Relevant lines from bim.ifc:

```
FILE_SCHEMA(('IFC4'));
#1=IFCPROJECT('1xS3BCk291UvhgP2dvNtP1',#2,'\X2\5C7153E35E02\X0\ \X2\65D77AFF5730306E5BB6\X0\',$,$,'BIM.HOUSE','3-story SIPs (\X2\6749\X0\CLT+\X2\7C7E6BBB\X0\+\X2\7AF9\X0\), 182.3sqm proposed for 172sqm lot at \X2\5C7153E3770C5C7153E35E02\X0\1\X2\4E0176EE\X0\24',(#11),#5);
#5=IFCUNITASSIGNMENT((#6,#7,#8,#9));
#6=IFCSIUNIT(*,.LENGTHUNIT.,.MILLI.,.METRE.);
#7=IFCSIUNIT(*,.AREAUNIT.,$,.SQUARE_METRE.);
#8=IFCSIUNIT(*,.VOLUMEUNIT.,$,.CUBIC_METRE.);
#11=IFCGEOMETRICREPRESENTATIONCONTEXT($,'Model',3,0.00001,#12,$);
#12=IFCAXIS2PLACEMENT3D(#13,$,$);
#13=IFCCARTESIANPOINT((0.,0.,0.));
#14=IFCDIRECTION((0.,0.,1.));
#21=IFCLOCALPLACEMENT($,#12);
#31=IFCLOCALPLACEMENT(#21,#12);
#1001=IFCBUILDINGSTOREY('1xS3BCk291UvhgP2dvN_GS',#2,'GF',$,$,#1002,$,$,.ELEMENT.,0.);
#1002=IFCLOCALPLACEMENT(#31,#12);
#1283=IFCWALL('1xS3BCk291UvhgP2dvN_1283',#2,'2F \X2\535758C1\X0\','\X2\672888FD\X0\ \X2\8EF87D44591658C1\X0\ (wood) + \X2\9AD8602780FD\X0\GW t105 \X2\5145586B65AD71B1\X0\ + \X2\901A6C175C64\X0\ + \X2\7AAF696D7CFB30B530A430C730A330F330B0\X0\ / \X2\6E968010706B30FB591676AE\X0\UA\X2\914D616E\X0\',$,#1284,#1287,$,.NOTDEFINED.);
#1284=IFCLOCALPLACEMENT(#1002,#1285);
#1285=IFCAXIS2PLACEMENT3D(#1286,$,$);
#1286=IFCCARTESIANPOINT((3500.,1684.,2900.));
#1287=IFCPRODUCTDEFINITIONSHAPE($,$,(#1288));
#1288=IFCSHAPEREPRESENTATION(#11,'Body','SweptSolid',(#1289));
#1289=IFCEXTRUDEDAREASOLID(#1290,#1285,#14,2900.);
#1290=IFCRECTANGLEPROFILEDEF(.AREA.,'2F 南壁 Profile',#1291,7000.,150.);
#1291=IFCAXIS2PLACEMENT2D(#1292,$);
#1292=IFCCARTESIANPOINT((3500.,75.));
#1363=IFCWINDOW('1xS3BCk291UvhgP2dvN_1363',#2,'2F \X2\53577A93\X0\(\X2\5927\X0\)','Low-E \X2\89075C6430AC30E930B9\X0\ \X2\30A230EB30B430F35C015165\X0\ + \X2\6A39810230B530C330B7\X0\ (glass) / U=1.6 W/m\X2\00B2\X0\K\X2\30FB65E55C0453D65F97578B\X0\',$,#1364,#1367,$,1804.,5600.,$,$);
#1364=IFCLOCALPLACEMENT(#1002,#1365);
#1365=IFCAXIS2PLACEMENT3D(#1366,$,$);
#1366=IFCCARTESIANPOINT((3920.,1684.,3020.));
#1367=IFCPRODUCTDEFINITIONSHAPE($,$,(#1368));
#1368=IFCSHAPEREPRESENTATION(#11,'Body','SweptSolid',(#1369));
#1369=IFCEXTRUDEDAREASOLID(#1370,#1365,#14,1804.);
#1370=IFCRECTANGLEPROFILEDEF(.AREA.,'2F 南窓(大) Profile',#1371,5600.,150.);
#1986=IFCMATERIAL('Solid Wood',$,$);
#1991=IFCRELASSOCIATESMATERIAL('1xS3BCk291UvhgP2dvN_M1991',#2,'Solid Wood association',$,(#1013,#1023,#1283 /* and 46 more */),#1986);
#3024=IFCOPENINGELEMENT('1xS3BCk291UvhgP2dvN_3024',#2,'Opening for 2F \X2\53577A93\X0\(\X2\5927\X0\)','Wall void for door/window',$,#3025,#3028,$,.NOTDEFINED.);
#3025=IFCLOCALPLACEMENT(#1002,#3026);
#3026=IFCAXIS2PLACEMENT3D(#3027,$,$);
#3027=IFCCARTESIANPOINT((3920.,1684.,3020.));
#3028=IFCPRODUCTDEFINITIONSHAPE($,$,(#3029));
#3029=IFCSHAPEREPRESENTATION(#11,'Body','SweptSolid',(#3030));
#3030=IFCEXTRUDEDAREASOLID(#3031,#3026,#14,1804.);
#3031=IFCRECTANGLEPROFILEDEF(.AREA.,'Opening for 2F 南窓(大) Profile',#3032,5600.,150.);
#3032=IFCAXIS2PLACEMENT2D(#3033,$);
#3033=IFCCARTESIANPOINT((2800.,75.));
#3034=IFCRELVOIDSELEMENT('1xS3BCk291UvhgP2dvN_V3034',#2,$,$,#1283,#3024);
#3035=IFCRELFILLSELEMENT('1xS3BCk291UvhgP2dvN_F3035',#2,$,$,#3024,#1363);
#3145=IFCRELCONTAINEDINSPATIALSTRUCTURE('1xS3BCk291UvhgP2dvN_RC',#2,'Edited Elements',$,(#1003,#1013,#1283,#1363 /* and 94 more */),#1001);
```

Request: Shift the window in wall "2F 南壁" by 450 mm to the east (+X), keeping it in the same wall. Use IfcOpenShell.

```python
import ifcopenshell
import ifcopenshell.api.geometry
import ifcopenshell.util.placement

model = ifcopenshell.open("bim.ifc")

window = model.by_guid("1xS3BCk291UvhgP2dvN_1363")
opening = window.FillsVoids[0].RelatingOpeningElement
wall = opening.VoidsElements[0].RelatingBuildingElement

wall_matrix = ifcopenshell.util.placement.get_local_placement(wall.ObjectPlacement)
shift = wall_matrix[:3, 0] * 450.0
before = ifcopenshell.util.placement.get_local_placement(window.ObjectPlacement)[:3, 3].copy()

# The window is not placed relative to its opening, so move both.
for product in (opening, window):
    matrix = ifcopenshell.util.placement.get_local_placement(product.ObjectPlacement)
    matrix[:3, 3] += shift
    ifcopenshell.api.geometry.edit_object_placement(model, product=product, matrix=matrix, is_si=False)

after = ifcopenshell.util.placement.get_local_placement(window.ObjectPlacement)[:3, 3]
print("window moved by", (after - before).round(3) + 0.0)

model.write("bim_edited.ifc")
```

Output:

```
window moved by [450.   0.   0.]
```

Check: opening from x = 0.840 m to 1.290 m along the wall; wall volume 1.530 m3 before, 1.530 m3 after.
